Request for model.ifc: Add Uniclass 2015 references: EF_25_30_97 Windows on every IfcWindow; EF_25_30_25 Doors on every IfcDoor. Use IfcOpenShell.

First a look at what the model holds.

```python
import ifcopenshell

model = ifcopenshell.open("model.ifc")
print(model.schema)
print("classifications:", [c.Name for c in model.by_type("IfcClassification")])
for ifc_class in ("IfcDoor", "IfcRoof", "IfcStair", "IfcWall", "IfcWindow"):
    print(ifc_class, len(model.by_type(ifc_class)))
```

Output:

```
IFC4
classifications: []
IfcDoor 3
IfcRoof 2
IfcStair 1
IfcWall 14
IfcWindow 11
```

```python
import ifcopenshell
import ifcopenshell.api.classification

model = ifcopenshell.open("model.ifc")

system = ifcopenshell.api.classification.add_classification(model, classification="Uniclass 2015")

codes = {
    "IfcWindow": ("EF_25_30_97", "Windows"),
    "IfcDoor": ("EF_25_30_25", "Doors"),
}
for ifc_class, (code, name) in codes.items():
    products = model.by_type(ifc_class)
    ifcopenshell.api.classification.add_reference(
        model, products=products, classification=system, identification=code, name=name
    )
    print(code, len(products))

model.write("model-out.ifc")
```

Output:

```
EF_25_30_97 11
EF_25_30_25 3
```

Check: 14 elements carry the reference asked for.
